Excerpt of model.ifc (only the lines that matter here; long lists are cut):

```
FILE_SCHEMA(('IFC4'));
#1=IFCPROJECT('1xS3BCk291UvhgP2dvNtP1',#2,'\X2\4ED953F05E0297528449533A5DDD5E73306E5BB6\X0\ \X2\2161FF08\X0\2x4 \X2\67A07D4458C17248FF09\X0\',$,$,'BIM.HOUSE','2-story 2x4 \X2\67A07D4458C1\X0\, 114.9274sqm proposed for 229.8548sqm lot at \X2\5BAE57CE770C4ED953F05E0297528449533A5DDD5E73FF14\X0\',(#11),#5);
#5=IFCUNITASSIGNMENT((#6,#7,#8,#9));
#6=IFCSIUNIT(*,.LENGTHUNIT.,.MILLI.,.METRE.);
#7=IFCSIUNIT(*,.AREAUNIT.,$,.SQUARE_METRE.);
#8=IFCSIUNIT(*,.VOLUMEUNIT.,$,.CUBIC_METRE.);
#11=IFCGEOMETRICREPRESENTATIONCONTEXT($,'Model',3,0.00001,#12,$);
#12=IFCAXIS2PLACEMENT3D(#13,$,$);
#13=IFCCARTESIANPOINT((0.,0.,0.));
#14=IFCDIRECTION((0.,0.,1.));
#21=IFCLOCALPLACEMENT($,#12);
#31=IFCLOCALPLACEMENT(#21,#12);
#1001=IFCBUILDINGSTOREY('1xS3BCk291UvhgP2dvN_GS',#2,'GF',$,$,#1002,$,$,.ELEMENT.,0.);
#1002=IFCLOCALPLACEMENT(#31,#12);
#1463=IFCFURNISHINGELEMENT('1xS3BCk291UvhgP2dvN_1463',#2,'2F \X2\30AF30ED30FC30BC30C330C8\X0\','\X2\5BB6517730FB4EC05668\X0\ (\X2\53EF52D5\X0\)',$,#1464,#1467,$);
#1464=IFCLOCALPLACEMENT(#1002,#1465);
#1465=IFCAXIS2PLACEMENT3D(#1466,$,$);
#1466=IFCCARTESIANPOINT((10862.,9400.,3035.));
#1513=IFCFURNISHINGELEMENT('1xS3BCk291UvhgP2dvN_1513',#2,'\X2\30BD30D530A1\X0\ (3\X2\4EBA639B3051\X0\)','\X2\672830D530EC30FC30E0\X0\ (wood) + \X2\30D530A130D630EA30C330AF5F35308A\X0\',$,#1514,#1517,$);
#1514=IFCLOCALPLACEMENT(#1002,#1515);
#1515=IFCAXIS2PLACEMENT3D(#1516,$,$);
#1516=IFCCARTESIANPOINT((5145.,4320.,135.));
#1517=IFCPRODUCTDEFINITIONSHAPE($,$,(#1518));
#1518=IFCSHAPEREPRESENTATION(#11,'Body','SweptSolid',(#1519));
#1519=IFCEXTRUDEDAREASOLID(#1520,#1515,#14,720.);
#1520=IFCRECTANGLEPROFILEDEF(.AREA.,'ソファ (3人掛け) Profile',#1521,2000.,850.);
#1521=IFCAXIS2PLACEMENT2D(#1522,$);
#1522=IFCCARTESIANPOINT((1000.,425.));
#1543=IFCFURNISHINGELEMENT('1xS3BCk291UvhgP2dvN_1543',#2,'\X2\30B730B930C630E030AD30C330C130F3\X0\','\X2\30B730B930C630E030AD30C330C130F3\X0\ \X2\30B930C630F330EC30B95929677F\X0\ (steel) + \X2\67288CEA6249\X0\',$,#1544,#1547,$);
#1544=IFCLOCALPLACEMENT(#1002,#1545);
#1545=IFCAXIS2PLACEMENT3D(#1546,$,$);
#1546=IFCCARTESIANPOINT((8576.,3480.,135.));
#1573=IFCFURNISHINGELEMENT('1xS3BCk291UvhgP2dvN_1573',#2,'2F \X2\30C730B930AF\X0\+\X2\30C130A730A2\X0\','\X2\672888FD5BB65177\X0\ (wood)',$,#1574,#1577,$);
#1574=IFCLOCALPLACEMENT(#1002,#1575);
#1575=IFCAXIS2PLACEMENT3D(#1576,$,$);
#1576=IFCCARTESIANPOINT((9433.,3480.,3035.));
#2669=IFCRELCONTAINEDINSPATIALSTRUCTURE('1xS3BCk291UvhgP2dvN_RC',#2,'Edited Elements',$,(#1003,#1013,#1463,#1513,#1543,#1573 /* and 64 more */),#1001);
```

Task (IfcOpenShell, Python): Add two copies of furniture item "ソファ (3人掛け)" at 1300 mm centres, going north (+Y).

```python
import numpy as np
import ifcopenshell
import ifcopenshell.api.geometry
import ifcopenshell.api.root
import ifcopenshell.util.element
import ifcopenshell.util.placement

model = ifcopenshell.open("model.ifc")


def reuse_history(source, copy):
    """copy_class also copies each property set's owner history, people and application; keep the originals."""
    for rel in copy.IsDefinedBy:
        if rel.is_a("IfcRelDefinesByProperties") and (history := rel.RelatingPropertyDefinition.OwnerHistory):
            rel.RelatingPropertyDefinition.OwnerHistory = source.OwnerHistory
            ifcopenshell.util.element.remove_deep2(model, history)


source = model.by_id(1513)
base = ifcopenshell.util.placement.get_local_placement(source.ObjectPlacement)
step = np.array([0.0, 1.0, 0.0]) * 1300.0

for i in range(1, 3):
    copy = ifcopenshell.api.root.copy_class(model, product=source)
    copy.Representation = ifcopenshell.util.element.copy_deep(
        model, source.Representation, exclude=["IfcGeometricRepresentationContext", "IfcRepresentationMap"]
    )
    reuse_history(source, copy)
    matrix = base.copy()
    matrix[:3, 3] += i * step
    print("added at", matrix[:3, 3].round(3) + 0.0)
    ifcopenshell.api.geometry.edit_object_placement(model, product=copy, matrix=matrix, is_si=False)

model.write("model_v2.ifc")
```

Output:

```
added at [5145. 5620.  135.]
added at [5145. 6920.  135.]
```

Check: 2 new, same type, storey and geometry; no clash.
